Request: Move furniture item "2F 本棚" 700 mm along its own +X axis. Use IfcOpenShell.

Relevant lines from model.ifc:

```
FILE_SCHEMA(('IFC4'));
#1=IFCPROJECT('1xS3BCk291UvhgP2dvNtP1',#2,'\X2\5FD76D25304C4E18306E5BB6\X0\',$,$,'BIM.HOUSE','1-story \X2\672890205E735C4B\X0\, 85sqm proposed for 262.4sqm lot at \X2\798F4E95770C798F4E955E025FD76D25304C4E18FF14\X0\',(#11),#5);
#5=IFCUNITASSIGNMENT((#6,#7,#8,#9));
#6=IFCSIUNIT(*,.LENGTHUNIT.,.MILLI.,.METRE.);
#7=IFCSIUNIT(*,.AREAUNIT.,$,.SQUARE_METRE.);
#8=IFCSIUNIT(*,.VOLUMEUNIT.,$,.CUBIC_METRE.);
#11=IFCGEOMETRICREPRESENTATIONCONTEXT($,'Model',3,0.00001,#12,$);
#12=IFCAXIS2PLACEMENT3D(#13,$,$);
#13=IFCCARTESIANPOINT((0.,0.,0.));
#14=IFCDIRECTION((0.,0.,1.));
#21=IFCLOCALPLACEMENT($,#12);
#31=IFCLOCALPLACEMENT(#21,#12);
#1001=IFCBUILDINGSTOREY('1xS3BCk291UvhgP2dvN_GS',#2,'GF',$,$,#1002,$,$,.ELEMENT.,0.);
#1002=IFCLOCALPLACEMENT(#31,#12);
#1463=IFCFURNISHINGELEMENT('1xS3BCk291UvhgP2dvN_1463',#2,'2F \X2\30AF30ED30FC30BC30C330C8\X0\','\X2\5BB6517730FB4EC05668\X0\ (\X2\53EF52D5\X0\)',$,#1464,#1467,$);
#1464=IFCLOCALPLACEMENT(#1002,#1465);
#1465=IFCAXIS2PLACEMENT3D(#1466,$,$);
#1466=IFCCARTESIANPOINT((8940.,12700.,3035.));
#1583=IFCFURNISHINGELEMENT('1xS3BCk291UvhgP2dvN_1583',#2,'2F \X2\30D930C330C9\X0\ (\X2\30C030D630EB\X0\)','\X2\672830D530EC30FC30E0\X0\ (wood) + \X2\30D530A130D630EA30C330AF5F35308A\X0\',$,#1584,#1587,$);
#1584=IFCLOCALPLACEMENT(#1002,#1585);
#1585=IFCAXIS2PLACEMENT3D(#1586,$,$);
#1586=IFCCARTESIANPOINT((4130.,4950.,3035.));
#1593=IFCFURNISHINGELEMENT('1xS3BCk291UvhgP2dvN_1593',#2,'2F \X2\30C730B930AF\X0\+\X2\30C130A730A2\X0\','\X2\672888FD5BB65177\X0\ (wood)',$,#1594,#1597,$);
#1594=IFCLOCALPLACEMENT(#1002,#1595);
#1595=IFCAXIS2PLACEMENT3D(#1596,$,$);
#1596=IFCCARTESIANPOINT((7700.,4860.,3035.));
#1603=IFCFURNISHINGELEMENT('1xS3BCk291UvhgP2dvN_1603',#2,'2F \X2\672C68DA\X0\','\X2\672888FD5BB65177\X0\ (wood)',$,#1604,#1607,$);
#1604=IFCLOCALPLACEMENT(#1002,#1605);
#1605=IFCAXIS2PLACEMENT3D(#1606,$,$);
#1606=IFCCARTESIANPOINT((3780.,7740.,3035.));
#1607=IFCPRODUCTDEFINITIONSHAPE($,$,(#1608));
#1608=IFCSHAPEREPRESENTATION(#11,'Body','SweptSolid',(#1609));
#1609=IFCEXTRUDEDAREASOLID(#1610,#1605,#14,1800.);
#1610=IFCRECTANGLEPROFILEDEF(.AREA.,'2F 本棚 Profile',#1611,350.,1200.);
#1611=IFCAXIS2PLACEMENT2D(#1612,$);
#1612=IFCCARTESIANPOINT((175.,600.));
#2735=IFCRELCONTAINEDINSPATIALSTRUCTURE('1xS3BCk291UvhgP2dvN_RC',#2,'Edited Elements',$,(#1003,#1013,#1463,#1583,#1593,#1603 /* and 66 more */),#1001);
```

```python
import ifcopenshell
import ifcopenshell.api.geometry
import ifcopenshell.util.placement
import ifcopenshell.util.unit

model = ifcopenshell.open("model.ifc")
unit_scale = ifcopenshell.util.unit.calculate_unit_scale(model)

item = model.by_guid("1xS3BCk291UvhgP2dvN_1603")
matrix = ifcopenshell.util.placement.get_local_placement(item.ObjectPlacement)
matrix[:3, 3] += matrix[:3, 0] * 0.7 / unit_scale
ifcopenshell.api.geometry.edit_object_placement(model, product=item, matrix=matrix, is_si=False)

print(ifcopenshell.util.placement.get_local_placement(item.ObjectPlacement).round(3) + 0.0)

model.write("model_v2.ifc")
```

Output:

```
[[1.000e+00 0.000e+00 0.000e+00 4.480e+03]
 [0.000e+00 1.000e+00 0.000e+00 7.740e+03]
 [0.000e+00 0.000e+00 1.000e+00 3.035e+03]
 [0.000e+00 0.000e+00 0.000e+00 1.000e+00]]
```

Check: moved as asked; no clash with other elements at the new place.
